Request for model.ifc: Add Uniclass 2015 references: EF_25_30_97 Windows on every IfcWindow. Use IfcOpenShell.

First a look at what the model holds.

```python
import ifcopenshell

model = ifcopenshell.open("model.ifc")
print(model.schema)
print("classifications:", [c.Name for c in model.by_type("IfcClassification")])
for ifc_class in ("IfcDoor", "IfcRoof", "IfcStair", "IfcWall", "IfcWindow"):
    print(ifc_class, len(model.by_type(ifc_class)))
```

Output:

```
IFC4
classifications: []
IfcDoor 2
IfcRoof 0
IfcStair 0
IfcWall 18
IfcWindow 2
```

```python
import ifcopenshell
import ifcopenshell.api.classification

model = ifcopenshell.open("model.ifc")

system = ifcopenshell.api.classification.add_classification(model, classification="Uniclass 2015")

codes = {
    "IfcWindow": ("EF_25_30_97", "Windows"),
}
for ifc_class, (code, name) in codes.items():
    products = model.by_type(ifc_class)
    ifcopenshell.api.classification.add_reference(
        model, products=products, classification=system, identification=code, name=name
    )
    print(code, len(products))

model.write("model_rev.ifc")
```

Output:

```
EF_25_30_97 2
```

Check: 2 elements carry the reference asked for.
